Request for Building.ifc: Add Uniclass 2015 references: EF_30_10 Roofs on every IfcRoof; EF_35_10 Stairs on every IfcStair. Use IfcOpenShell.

First a look at what the model holds.

```python
import ifcopenshell

model = ifcopenshell.open("Building.ifc")
print(model.schema)
print("classifications:", [c.Name for c in model.by_type("IfcClassification")])
for ifc_class in ("IfcDoor", "IfcRoof", "IfcStair", "IfcWall", "IfcWindow"):
    print(ifc_class, len(model.by_type(ifc_class)))
```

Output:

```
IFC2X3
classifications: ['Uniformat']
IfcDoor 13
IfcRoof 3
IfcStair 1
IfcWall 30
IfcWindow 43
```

```python
import ifcopenshell
import ifcopenshell.api.classification

model = ifcopenshell.open("Building.ifc")

# IFC2X3 requires Source and Edition and has no link from the project to the system.
system = model.create_entity("IfcClassification", Source="NBS", Edition="2015", Name="Uniclass 2015")

codes = {
    "IfcRoof": ("EF_30_10", "Roofs"),
    "IfcStair": ("EF_35_10", "Stairs"),
}
for ifc_class, (code, name) in codes.items():
    products = model.by_type(ifc_class)
    ifcopenshell.api.classification.add_reference(
        model, products=products, classification=system, identification=code, name=name
    )
    print(code, len(products))

model.write("Building_rev.ifc")
```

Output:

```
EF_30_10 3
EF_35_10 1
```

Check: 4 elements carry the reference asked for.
